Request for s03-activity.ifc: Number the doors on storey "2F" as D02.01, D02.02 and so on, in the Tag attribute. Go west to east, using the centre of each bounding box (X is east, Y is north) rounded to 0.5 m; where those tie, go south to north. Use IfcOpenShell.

First a look at what the model holds.

```python
import ifcopenshell
import ifcopenshell.util.element
import ifcopenshell.util.placement

model = ifcopenshell.open("s03-activity.ifc")
print(model.schema)
storey = next(s for s in model.by_type("IfcBuildingStorey") if s.Name == "2F")
doors = [e for e in ifcopenshell.util.element.get_decomposition(storey) if e.is_a("IfcDoor")]
for e in sorted(doors, key=lambda e: e.id()):
    origin = ifcopenshell.util.placement.get_local_placement(e.ObjectPlacement)[:3, 3]
    print(e.id(), e.Tag, e.Name, origin.round(2) + 0.0, sep=" | ")
```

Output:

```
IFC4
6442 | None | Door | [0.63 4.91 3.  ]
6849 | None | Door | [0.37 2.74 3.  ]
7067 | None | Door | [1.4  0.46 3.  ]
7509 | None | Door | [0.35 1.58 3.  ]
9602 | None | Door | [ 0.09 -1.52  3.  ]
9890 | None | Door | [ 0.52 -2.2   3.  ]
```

```python
import ifcopenshell
import ifcopenshell.geom
import ifcopenshell.util.element
import ifcopenshell.util.shape

model = ifcopenshell.open("s03-activity.ifc")
settings = ifcopenshell.geom.settings()
settings.set("use-world-coords", True)


def centre(element):
    shape = ifcopenshell.geom.create_shape(settings, element)
    return ifcopenshell.util.shape.get_bbox_centroid(shape.geometry)


storey = next(s for s in model.by_type("IfcBuildingStorey") if s.Name == "2F")
doors = [e for e in ifcopenshell.util.element.get_decomposition(storey) if e.is_a("IfcDoor")]

# Insertion points can sit at a corner or the storey origin, so sort by the geometry (in metres).
centres = {e: centre(e) for e in doors}
doors.sort(key=lambda e: (round(centres[e][0] / 0.5), centres[e][1]))

for i, e in enumerate(doors, start=1):
    number = f"D02.{i:02d}"
    e.Tag = number
    print(e.id(), number)

model.write("s03-activity_edited.ifc")
```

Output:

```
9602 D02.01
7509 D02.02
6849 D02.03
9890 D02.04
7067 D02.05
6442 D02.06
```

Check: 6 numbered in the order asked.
